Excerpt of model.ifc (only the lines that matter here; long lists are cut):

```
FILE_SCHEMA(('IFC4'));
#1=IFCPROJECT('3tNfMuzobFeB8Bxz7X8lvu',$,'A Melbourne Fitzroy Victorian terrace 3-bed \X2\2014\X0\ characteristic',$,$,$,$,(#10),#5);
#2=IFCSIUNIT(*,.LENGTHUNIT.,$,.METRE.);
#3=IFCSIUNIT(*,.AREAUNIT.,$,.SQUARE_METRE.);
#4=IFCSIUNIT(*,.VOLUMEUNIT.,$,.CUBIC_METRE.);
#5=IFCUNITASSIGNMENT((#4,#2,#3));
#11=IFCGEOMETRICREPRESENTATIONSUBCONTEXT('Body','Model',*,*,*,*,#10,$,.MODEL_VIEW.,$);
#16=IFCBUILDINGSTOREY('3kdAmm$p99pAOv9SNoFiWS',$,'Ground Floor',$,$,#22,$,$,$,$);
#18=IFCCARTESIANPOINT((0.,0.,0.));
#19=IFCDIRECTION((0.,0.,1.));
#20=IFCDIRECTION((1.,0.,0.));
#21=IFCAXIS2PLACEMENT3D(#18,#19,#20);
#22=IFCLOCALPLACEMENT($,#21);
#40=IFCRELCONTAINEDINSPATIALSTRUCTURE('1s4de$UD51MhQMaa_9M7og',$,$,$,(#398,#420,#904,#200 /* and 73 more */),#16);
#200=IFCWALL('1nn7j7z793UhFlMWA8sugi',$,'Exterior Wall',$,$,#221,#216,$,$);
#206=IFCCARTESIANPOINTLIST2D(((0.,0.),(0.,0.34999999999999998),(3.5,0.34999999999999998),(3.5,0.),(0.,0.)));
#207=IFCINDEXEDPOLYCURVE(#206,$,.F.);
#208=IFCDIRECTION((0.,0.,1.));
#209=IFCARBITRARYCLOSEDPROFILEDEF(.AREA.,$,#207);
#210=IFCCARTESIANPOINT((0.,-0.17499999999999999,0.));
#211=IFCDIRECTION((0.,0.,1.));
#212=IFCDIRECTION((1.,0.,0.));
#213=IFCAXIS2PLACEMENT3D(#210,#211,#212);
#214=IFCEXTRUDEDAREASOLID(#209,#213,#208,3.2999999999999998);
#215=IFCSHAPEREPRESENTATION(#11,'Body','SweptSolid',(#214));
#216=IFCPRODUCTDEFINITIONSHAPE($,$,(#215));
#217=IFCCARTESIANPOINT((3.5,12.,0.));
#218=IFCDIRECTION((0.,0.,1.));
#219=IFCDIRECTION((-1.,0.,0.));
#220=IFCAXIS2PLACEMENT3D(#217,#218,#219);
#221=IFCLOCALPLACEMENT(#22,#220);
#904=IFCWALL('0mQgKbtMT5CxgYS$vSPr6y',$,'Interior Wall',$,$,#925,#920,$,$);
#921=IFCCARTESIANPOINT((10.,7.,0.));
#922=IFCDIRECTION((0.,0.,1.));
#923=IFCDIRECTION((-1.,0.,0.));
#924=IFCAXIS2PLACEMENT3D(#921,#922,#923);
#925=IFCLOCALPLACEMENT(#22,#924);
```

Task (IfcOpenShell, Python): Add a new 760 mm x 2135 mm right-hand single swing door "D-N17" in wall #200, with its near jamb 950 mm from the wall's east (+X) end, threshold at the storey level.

```python
import numpy as np
import ifcopenshell
import ifcopenshell.api.feature
import ifcopenshell.api.geometry
import ifcopenshell.api.root
import ifcopenshell.api.spatial
import ifcopenshell.geom
import ifcopenshell.util.element
import ifcopenshell.util.placement
import ifcopenshell.util.representation
import ifcopenshell.util.shape
import ifcopenshell.util.unit

model = ifcopenshell.open("model.ifc")
unit_scale = ifcopenshell.util.unit.calculate_unit_scale(model)
settings = ifcopenshell.geom.settings()


def volume(element):
    """Net volume in cubic metres, openings subtracted."""
    shape = ifcopenshell.geom.create_shape(settings, element)
    return ifcopenshell.util.shape.get_volume(shape.geometry)


wall = model.by_guid("1nn7j7z793UhFlMWA8sugi")
storey = ifcopenshell.util.element.get_container(wall, ifc_class="IfcBuildingStorey")
context = ifcopenshell.util.representation.get_context(model, "Model", "Body", "MODEL_VIEW")
before = volume(wall)

width, height, from_end, sill = 0.76, 2.135, 0.95, 0.0  # metres

# The wall runs along its own X axis, and the end named is its -X end.
wall_shape = ifcopenshell.geom.create_shape(settings, wall)
x, y, z = ifcopenshell.util.shape.get_vertices(wall_shape.geometry).T
start = x.min() + from_end
face, thickness = float(y.min()), float(y.max() - y.min())
wall_matrix = ifcopenshell.util.placement.get_local_placement(wall.ObjectPlacement)
level = ifcopenshell.util.placement.get_local_placement(storey.ObjectPlacement)[2, 3]


def in_wall(x, y):
    """Placement at x, y metres in the wall's axes, at sill height."""
    matrix = wall_matrix.copy()
    matrix[:, 3] = wall_matrix @ np.array([x / unit_scale, y / unit_scale, 0.0, 1.0])
    matrix[2, 3] = level + sill / unit_scale
    return matrix


# Opening: a box that overshoots both wall faces by 50 mm.
opening = ifcopenshell.api.root.create_entity(model, ifc_class="IfcOpeningElement", predefined_type="OPENING")
box = ifcopenshell.api.geometry.add_wall_representation(
    model, context=context, length=width, height=height, thickness=thickness + 0.1
)
ifcopenshell.api.geometry.assign_representation(model, product=opening, representation=box)
ifcopenshell.api.geometry.edit_object_placement(model, product=opening, matrix=in_wall(start, face - 0.05), is_si=False)
ifcopenshell.api.feature.add_feature(model, feature=opening, element=wall)

door = ifcopenshell.api.root.create_entity(model, ifc_class="IfcDoor", name="D-N17", predefined_type="DOOR")
door.OverallWidth, door.OverallHeight = width / unit_scale, height / unit_scale
door.OperationType = "SINGLE_SWING_RIGHT"
body = ifcopenshell.api.geometry.add_door_representation(
    model,
    context=context,
    overall_width=door.OverallWidth,
    overall_height=door.OverallHeight,
    operation_type="SINGLE_SWING_RIGHT",
    lining_properties={"LiningDepth": thickness / unit_scale, "ThresholdDepth": thickness / unit_scale},
)
ifcopenshell.api.geometry.assign_representation(model, product=door, representation=body)
ifcopenshell.api.spatial.assign_container(model, products=[door], relating_structure=storey)
ifcopenshell.api.feature.add_filling(model, opening=opening, element=door)

# The lining spans the wall, so the door starts at the wall face.
ifcopenshell.api.geometry.edit_object_placement(model, product=door, matrix=in_wall(start, face), is_si=False)

after = volume(wall)

print(f"wall volume {before:.3f} -> {after:.3f} m3")

model.write("model_v2.ifc")
```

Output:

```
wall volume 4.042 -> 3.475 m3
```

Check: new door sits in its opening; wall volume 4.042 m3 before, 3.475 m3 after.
